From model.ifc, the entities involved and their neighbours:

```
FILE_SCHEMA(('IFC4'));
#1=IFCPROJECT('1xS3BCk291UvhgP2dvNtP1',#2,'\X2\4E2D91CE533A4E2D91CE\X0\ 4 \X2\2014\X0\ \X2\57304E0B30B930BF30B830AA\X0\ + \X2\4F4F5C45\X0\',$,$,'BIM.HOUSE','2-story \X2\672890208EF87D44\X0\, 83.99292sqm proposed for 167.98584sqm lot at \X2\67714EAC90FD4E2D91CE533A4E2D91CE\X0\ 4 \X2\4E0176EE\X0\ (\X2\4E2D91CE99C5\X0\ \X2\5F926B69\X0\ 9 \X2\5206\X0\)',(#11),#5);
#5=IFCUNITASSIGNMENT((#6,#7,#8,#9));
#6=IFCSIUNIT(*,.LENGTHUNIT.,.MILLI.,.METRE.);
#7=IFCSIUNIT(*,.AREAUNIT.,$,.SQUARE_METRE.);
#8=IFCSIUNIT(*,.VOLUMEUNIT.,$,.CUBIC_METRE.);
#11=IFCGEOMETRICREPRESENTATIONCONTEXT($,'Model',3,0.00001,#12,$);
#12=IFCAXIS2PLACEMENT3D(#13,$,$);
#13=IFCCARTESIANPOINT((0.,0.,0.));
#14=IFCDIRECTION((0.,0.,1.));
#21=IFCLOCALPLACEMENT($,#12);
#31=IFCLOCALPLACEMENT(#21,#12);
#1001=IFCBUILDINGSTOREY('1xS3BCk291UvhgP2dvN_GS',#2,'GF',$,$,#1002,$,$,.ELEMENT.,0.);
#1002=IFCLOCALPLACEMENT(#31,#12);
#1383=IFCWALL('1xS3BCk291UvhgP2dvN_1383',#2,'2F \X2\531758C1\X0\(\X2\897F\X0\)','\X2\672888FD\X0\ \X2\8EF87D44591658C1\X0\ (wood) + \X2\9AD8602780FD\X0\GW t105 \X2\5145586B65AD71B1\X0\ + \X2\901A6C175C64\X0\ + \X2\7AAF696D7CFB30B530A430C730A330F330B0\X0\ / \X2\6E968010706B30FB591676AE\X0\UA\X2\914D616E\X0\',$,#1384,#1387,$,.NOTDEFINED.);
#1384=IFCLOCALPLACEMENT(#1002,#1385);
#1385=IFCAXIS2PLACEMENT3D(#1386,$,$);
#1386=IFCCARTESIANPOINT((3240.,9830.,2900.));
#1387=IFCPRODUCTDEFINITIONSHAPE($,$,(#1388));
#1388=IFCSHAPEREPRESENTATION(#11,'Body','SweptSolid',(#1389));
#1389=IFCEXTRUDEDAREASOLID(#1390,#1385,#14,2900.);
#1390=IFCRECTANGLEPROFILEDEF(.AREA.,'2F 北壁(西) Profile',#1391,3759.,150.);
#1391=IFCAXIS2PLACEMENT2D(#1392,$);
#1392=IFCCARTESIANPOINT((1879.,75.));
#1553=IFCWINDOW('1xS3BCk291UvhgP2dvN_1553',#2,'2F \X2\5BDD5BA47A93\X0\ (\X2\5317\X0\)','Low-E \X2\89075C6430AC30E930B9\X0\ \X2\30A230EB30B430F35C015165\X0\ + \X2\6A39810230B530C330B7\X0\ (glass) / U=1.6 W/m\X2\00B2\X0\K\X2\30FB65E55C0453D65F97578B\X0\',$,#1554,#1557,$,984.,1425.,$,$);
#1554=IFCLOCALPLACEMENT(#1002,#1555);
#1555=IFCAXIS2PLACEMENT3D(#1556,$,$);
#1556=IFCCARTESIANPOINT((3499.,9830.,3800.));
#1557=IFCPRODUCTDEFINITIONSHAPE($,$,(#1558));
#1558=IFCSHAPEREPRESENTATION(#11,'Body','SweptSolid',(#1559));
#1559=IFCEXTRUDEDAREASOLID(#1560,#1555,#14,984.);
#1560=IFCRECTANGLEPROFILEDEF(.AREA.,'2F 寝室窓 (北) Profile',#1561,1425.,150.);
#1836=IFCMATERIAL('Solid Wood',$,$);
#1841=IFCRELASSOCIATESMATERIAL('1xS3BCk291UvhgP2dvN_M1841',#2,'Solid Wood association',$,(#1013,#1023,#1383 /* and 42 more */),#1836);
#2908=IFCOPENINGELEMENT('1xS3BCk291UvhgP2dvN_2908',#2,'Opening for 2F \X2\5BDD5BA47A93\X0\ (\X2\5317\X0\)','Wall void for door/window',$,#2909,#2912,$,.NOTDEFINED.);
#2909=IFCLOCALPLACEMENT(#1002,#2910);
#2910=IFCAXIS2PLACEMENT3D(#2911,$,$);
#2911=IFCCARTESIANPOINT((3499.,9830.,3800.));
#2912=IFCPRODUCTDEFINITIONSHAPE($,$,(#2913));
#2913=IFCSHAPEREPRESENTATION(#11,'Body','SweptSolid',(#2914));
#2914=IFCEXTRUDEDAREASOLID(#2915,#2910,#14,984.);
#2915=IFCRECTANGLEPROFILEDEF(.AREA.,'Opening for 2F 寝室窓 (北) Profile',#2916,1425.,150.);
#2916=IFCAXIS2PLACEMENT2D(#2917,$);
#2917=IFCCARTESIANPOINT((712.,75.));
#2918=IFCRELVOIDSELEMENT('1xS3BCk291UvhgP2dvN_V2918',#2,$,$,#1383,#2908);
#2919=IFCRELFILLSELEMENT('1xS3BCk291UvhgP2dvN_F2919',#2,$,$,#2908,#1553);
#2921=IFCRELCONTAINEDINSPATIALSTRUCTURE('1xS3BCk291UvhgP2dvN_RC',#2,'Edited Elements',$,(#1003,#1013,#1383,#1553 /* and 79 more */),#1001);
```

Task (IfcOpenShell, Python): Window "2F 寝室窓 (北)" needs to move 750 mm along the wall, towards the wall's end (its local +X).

```python
import ifcopenshell
import ifcopenshell.api.geometry
import ifcopenshell.util.placement
import ifcopenshell.util.unit

model = ifcopenshell.open("model.ifc")
unit_scale = ifcopenshell.util.unit.calculate_unit_scale(model)

window = model.by_guid("1xS3BCk291UvhgP2dvN_1553")
opening = window.FillsVoids[0].RelatingOpeningElement
wall = opening.VoidsElements[0].RelatingBuildingElement

wall_matrix = ifcopenshell.util.placement.get_local_placement(wall.ObjectPlacement)
shift = wall_matrix[:3, 0] * 0.75 / unit_scale
before = ifcopenshell.util.placement.get_local_placement(window.ObjectPlacement)[:3, 3].copy()

# The window is not placed relative to its opening, so move both.
for product in (opening, window):
    matrix = ifcopenshell.util.placement.get_local_placement(product.ObjectPlacement)
    matrix[:3, 3] += shift
    ifcopenshell.api.geometry.edit_object_placement(model, product=product, matrix=matrix, is_si=False)

after = ifcopenshell.util.placement.get_local_placement(window.ObjectPlacement)[:3, 3]
print("window moved by", (after - before).round(3) + 0.0)

model.write("model_edited.ifc")
```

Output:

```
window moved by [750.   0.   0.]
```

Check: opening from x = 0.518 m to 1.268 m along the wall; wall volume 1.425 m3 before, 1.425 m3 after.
